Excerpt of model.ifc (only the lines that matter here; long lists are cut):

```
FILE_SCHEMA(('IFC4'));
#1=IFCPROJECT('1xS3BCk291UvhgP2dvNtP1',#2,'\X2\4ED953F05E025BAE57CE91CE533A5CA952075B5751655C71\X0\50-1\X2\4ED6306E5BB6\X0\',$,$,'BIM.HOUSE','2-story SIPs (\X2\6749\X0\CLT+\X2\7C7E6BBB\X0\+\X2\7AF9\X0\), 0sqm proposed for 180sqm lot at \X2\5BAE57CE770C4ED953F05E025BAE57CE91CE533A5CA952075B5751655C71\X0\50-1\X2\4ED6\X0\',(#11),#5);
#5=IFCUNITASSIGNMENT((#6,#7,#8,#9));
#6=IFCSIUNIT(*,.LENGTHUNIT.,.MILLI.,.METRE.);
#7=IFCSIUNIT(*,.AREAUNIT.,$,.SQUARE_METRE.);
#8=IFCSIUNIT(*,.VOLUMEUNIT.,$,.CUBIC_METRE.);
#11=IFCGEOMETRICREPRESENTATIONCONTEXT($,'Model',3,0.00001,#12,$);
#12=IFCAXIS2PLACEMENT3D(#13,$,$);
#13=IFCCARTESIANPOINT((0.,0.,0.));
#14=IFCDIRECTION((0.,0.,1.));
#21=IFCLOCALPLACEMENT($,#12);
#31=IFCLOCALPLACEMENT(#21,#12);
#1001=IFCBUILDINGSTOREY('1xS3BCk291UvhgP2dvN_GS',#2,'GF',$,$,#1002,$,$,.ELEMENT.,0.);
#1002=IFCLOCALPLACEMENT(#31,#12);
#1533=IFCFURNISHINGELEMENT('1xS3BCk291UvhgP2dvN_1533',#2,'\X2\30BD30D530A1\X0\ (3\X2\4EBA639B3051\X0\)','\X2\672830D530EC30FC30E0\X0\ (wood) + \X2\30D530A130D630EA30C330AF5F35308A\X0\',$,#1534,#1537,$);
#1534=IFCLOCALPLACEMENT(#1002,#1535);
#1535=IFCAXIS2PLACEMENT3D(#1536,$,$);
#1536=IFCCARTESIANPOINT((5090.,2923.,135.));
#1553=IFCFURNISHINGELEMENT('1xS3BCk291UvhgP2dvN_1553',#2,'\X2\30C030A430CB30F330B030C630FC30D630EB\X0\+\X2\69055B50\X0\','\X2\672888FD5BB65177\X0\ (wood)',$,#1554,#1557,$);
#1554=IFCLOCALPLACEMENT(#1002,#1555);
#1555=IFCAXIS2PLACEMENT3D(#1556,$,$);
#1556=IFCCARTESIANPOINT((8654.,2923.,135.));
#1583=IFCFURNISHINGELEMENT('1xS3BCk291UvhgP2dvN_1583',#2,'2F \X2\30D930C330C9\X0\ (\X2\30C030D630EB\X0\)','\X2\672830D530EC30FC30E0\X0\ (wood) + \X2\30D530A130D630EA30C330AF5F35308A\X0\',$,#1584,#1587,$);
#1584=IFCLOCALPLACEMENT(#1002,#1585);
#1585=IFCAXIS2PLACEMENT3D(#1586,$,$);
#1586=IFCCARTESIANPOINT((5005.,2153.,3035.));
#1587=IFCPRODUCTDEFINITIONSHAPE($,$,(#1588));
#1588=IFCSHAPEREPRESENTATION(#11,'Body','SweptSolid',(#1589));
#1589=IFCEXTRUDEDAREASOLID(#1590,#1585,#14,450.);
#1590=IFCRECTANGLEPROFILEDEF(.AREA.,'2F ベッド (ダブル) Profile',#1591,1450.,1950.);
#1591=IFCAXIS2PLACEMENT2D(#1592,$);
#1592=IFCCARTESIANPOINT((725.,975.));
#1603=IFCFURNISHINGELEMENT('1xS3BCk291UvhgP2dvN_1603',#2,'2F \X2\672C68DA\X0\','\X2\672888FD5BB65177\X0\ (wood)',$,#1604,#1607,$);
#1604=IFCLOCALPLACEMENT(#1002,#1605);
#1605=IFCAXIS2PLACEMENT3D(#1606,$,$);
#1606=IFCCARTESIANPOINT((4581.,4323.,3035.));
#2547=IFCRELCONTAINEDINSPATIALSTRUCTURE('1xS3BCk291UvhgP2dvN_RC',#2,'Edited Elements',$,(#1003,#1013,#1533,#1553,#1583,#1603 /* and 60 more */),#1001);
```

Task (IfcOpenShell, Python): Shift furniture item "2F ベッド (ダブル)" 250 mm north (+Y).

```python
import ifcopenshell
import ifcopenshell.api.geometry
import ifcopenshell.util.placement
import ifcopenshell.util.unit

model = ifcopenshell.open("model.ifc")
unit_scale = ifcopenshell.util.unit.calculate_unit_scale(model)

item = model.by_id(1583)
matrix = ifcopenshell.util.placement.get_local_placement(item.ObjectPlacement)
matrix[1, 3] += 0.25 / unit_scale
ifcopenshell.api.geometry.edit_object_placement(model, product=item, matrix=matrix, is_si=False)

print(ifcopenshell.util.placement.get_local_placement(item.ObjectPlacement).round(3) + 0.0)

model.write("model_v2.ifc")
```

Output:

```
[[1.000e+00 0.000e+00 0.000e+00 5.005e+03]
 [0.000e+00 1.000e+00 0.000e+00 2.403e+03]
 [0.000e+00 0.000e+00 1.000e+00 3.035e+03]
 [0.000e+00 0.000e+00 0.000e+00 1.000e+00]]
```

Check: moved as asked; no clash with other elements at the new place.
